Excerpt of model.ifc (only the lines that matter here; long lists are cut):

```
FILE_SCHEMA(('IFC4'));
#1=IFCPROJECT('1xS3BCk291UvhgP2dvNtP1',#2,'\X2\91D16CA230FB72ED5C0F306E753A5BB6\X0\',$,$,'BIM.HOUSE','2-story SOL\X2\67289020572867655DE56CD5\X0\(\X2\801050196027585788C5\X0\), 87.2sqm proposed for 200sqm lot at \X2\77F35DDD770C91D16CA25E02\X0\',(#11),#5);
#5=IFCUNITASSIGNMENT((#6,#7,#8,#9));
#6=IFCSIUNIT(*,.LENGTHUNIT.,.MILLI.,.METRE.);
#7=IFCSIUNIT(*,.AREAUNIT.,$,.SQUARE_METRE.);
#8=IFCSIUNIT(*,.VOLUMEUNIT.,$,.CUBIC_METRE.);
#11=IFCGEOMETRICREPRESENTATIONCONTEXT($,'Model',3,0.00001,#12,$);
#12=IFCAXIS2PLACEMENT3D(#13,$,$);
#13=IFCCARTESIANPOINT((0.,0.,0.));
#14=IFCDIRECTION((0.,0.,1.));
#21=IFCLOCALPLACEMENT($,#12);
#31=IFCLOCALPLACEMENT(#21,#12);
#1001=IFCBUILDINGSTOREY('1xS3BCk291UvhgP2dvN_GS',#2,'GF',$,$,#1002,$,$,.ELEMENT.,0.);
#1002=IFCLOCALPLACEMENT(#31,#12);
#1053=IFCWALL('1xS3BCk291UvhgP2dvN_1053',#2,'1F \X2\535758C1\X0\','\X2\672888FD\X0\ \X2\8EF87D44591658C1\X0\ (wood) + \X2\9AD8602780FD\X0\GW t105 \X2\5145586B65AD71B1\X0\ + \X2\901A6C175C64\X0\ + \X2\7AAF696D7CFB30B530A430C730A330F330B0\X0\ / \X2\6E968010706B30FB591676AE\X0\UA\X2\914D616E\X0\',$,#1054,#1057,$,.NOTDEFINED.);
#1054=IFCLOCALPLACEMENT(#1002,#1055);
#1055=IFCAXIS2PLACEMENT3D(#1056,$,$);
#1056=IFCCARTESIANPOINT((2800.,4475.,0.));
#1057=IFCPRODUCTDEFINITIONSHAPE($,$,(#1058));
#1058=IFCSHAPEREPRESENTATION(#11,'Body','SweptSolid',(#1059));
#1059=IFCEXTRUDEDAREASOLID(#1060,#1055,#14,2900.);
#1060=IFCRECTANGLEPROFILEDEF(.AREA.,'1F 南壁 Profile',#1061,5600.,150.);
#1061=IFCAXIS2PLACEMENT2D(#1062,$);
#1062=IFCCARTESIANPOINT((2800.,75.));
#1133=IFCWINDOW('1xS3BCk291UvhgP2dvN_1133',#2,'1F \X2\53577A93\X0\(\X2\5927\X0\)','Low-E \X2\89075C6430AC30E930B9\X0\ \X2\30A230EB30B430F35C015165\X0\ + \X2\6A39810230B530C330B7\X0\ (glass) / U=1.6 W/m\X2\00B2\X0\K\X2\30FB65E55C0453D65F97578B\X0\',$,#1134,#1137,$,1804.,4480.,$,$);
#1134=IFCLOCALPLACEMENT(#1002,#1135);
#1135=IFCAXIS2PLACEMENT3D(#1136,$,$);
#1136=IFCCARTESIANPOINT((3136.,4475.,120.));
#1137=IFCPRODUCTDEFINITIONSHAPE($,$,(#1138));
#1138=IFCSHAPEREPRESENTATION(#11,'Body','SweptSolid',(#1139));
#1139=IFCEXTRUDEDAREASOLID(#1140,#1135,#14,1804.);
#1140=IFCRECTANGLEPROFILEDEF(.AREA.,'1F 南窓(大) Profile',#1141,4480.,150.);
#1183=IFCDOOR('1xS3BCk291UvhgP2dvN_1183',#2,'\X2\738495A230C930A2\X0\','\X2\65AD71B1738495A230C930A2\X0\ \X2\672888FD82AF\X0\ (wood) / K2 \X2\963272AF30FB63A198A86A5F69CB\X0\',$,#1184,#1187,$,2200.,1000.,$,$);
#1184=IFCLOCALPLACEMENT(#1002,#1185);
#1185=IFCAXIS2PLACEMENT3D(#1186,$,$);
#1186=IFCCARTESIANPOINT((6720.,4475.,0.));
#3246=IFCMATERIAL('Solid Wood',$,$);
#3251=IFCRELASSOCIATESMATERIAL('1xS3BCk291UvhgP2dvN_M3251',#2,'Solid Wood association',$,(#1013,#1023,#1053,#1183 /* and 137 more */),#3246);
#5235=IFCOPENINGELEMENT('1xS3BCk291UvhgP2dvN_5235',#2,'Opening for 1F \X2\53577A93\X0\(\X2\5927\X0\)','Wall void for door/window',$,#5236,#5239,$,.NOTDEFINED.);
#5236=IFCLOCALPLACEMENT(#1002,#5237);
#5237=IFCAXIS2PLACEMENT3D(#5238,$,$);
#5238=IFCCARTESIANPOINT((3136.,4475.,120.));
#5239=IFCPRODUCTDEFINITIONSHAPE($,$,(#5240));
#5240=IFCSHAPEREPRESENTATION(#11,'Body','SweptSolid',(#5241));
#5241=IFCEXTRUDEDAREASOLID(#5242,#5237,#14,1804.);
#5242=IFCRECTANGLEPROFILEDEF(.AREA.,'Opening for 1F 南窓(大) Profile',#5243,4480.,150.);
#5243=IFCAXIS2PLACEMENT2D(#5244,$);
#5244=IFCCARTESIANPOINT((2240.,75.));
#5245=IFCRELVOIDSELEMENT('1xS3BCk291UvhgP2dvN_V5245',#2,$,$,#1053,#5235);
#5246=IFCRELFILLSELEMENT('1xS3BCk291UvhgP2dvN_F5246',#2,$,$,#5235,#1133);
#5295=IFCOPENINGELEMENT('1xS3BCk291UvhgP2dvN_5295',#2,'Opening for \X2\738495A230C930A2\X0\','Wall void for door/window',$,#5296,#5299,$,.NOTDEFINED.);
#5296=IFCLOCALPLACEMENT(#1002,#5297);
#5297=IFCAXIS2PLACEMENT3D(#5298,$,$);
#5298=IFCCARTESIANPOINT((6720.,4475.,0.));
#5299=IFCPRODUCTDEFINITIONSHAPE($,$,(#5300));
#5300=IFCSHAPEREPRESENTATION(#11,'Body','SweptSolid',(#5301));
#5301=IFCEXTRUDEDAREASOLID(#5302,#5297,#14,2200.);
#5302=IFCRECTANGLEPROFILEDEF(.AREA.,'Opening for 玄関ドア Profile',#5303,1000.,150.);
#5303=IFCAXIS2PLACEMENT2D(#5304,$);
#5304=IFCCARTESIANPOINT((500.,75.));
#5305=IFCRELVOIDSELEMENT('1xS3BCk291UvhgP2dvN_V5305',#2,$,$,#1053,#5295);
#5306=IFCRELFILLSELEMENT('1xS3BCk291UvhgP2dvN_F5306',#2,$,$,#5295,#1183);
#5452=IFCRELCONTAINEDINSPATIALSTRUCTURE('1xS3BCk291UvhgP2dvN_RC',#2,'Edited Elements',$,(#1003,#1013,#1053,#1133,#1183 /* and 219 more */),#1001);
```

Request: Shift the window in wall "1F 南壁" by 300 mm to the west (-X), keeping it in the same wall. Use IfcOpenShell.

```python
import ifcopenshell
import ifcopenshell.api.geometry
import ifcopenshell.util.placement
import ifcopenshell.util.unit

model = ifcopenshell.open("model.ifc")
unit_scale = ifcopenshell.util.unit.calculate_unit_scale(model)

window = model.by_guid("1xS3BCk291UvhgP2dvN_1133")
opening = window.FillsVoids[0].RelatingOpeningElement
wall = opening.VoidsElements[0].RelatingBuildingElement

wall_matrix = ifcopenshell.util.placement.get_local_placement(wall.ObjectPlacement)
shift = wall_matrix[:3, 0] * -0.3 / unit_scale
before = ifcopenshell.util.placement.get_local_placement(window.ObjectPlacement)[:3, 3].copy()

# The window is not placed relative to its opening, so move both.
for product in (opening, window):
    matrix = ifcopenshell.util.placement.get_local_placement(product.ObjectPlacement)
    matrix[:3, 3] += shift
    ifcopenshell.api.geometry.edit_object_placement(model, product=product, matrix=matrix, is_si=False)

after = ifcopenshell.util.placement.get_local_placement(window.ObjectPlacement)[:3, 3]
print("window moved by", (after - before).round(3) + 0.0)

model.write("model-out.ifc")
```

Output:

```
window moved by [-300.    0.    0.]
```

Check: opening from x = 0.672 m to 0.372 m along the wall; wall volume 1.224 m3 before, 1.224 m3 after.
